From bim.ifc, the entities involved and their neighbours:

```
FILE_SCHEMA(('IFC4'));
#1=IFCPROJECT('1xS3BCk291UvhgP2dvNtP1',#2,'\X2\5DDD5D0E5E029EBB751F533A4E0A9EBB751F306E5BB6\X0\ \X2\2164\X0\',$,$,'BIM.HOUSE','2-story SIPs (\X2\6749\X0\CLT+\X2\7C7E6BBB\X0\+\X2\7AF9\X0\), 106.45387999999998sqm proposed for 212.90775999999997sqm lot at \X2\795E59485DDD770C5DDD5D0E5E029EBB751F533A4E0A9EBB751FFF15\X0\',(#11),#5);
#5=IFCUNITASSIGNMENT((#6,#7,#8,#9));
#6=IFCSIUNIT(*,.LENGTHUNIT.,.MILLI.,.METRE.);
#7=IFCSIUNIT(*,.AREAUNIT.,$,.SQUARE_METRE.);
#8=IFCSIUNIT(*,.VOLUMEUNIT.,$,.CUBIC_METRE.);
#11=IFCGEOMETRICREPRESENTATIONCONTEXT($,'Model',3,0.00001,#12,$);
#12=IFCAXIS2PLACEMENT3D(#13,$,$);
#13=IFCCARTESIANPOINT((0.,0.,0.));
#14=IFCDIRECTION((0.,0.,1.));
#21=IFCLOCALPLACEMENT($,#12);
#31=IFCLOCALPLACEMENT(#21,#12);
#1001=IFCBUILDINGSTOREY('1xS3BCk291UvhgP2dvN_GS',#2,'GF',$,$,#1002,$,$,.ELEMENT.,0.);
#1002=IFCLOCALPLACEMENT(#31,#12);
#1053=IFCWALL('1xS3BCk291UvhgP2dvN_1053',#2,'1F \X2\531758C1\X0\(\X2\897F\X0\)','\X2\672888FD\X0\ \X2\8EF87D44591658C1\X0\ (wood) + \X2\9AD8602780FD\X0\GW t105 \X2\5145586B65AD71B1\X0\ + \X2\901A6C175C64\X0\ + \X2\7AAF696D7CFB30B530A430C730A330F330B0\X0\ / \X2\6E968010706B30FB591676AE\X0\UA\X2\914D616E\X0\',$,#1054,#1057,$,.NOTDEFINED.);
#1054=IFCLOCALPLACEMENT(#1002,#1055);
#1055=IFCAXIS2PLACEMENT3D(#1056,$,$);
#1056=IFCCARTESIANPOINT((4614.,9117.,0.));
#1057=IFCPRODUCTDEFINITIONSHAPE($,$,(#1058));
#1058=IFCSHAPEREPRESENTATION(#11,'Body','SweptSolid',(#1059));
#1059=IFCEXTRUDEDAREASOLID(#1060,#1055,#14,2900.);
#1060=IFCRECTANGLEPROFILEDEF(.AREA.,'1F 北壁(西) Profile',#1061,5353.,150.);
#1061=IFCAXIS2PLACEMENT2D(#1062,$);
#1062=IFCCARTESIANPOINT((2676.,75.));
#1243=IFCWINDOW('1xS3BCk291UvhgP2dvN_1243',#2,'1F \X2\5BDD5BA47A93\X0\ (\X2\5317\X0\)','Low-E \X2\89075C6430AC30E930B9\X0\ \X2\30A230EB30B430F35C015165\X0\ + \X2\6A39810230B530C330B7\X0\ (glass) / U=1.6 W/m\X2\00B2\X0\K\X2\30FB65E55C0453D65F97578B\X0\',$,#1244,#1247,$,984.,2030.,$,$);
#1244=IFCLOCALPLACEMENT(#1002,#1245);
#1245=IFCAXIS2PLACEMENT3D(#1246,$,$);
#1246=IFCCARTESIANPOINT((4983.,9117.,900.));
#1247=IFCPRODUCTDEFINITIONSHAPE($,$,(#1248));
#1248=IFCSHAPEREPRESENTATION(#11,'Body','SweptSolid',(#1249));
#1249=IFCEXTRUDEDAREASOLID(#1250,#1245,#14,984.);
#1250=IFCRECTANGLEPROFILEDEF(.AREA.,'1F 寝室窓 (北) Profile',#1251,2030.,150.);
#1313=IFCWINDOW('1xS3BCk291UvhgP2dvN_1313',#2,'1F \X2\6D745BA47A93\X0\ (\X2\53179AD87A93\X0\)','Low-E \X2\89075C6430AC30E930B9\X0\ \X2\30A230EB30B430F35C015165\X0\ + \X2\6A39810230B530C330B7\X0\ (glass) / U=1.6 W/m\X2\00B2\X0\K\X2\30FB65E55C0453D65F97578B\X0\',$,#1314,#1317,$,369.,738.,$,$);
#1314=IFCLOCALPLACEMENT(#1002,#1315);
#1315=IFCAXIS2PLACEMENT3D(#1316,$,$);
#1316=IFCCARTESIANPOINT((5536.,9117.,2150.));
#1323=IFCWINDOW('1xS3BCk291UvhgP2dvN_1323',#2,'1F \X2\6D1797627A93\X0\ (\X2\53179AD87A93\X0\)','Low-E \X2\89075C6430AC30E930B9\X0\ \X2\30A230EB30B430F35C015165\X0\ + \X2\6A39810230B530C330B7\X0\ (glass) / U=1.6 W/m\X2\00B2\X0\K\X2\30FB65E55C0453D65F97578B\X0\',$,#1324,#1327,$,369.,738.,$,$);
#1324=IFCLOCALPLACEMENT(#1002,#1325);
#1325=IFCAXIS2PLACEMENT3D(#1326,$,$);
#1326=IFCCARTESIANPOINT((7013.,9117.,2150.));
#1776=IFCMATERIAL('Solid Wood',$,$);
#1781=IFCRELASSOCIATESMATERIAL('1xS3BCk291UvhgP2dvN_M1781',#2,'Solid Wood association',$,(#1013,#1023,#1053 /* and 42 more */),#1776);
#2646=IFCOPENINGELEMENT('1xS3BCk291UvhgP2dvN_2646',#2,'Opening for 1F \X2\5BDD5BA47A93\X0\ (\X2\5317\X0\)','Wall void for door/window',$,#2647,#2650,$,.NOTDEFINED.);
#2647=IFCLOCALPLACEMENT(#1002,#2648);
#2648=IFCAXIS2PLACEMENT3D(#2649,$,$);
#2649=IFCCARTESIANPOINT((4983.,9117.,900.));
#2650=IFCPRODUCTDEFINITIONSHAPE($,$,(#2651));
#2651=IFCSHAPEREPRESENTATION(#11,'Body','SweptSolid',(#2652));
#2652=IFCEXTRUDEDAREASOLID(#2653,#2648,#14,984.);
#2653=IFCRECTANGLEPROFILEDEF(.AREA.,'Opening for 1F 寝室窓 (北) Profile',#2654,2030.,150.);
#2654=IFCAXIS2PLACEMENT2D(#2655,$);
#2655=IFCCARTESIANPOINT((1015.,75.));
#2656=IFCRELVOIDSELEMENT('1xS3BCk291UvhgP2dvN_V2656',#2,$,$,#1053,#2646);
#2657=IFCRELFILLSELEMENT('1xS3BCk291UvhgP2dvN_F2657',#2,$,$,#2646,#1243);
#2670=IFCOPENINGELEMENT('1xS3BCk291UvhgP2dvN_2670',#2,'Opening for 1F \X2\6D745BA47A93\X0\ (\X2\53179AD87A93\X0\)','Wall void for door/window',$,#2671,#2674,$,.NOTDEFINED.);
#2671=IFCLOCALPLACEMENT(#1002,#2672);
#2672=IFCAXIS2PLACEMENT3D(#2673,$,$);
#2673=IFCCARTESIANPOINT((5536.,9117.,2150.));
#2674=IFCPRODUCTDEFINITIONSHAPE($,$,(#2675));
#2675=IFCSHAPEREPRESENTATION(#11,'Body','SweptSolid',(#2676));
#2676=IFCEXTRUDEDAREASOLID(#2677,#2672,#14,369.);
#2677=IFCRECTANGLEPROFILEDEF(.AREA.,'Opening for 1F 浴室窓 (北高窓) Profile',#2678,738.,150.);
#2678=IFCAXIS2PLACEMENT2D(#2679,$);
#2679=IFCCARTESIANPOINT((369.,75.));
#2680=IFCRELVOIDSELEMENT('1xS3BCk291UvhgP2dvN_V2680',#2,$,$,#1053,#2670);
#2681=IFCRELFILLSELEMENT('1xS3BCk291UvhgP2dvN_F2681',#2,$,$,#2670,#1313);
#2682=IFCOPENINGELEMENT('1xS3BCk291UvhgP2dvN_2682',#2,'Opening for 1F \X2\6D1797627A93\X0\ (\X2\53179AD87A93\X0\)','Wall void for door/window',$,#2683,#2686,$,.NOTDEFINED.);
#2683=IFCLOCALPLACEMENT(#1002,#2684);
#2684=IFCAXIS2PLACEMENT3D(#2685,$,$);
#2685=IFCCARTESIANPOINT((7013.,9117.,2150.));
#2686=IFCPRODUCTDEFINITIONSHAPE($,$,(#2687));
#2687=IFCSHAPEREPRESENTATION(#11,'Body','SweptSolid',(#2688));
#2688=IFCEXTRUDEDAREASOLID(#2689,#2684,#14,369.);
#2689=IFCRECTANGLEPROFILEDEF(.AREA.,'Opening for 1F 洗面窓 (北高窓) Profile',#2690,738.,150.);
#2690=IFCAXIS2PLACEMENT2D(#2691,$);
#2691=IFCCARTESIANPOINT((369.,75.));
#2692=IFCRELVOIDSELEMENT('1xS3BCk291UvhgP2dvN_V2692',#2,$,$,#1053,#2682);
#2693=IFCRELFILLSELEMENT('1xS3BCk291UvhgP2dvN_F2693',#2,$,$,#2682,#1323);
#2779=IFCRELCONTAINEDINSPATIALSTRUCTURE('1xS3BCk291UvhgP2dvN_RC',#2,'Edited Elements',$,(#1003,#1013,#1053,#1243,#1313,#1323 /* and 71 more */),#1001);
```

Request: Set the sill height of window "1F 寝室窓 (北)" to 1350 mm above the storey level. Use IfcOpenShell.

```python
import numpy as np
import ifcopenshell
import ifcopenshell.api.geometry
import ifcopenshell.geom
import ifcopenshell.util.element
import ifcopenshell.util.placement
import ifcopenshell.util.shape
import ifcopenshell.util.unit

model = ifcopenshell.open("bim.ifc")
unit_scale = ifcopenshell.util.unit.calculate_unit_scale(model)

window = model.by_id(1243)
opening = window.FillsVoids[0].RelatingOpeningElement
storey = ifcopenshell.util.element.get_container(window, ifc_class="IfcBuildingStorey")
level = ifcopenshell.util.placement.get_local_placement(storey.ObjectPlacement)[2, 3]

# The opening's origin need not be at the sill, so measure its lowest point.
shape = ifcopenshell.geom.create_shape(ifcopenshell.geom.settings(), opening)
bottom = ifcopenshell.util.shape.get_shape_bottom_elevation(shape, shape.geometry) / unit_scale
dz = level + 1.35 / unit_scale - bottom

shift = np.array([0.0, 0.0, dz])
# The window is not placed relative to its opening, so move both.
for product in (opening, window):
    matrix = ifcopenshell.util.placement.get_local_placement(product.ObjectPlacement)
    matrix[:3, 3] += shift
    ifcopenshell.api.geometry.edit_object_placement(model, product=product, matrix=matrix, is_si=False)

print(f"moved by {dz * unit_scale:+.3f} m")

model.write("bim_updated.ifc")
```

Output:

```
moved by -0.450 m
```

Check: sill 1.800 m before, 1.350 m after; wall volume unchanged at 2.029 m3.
